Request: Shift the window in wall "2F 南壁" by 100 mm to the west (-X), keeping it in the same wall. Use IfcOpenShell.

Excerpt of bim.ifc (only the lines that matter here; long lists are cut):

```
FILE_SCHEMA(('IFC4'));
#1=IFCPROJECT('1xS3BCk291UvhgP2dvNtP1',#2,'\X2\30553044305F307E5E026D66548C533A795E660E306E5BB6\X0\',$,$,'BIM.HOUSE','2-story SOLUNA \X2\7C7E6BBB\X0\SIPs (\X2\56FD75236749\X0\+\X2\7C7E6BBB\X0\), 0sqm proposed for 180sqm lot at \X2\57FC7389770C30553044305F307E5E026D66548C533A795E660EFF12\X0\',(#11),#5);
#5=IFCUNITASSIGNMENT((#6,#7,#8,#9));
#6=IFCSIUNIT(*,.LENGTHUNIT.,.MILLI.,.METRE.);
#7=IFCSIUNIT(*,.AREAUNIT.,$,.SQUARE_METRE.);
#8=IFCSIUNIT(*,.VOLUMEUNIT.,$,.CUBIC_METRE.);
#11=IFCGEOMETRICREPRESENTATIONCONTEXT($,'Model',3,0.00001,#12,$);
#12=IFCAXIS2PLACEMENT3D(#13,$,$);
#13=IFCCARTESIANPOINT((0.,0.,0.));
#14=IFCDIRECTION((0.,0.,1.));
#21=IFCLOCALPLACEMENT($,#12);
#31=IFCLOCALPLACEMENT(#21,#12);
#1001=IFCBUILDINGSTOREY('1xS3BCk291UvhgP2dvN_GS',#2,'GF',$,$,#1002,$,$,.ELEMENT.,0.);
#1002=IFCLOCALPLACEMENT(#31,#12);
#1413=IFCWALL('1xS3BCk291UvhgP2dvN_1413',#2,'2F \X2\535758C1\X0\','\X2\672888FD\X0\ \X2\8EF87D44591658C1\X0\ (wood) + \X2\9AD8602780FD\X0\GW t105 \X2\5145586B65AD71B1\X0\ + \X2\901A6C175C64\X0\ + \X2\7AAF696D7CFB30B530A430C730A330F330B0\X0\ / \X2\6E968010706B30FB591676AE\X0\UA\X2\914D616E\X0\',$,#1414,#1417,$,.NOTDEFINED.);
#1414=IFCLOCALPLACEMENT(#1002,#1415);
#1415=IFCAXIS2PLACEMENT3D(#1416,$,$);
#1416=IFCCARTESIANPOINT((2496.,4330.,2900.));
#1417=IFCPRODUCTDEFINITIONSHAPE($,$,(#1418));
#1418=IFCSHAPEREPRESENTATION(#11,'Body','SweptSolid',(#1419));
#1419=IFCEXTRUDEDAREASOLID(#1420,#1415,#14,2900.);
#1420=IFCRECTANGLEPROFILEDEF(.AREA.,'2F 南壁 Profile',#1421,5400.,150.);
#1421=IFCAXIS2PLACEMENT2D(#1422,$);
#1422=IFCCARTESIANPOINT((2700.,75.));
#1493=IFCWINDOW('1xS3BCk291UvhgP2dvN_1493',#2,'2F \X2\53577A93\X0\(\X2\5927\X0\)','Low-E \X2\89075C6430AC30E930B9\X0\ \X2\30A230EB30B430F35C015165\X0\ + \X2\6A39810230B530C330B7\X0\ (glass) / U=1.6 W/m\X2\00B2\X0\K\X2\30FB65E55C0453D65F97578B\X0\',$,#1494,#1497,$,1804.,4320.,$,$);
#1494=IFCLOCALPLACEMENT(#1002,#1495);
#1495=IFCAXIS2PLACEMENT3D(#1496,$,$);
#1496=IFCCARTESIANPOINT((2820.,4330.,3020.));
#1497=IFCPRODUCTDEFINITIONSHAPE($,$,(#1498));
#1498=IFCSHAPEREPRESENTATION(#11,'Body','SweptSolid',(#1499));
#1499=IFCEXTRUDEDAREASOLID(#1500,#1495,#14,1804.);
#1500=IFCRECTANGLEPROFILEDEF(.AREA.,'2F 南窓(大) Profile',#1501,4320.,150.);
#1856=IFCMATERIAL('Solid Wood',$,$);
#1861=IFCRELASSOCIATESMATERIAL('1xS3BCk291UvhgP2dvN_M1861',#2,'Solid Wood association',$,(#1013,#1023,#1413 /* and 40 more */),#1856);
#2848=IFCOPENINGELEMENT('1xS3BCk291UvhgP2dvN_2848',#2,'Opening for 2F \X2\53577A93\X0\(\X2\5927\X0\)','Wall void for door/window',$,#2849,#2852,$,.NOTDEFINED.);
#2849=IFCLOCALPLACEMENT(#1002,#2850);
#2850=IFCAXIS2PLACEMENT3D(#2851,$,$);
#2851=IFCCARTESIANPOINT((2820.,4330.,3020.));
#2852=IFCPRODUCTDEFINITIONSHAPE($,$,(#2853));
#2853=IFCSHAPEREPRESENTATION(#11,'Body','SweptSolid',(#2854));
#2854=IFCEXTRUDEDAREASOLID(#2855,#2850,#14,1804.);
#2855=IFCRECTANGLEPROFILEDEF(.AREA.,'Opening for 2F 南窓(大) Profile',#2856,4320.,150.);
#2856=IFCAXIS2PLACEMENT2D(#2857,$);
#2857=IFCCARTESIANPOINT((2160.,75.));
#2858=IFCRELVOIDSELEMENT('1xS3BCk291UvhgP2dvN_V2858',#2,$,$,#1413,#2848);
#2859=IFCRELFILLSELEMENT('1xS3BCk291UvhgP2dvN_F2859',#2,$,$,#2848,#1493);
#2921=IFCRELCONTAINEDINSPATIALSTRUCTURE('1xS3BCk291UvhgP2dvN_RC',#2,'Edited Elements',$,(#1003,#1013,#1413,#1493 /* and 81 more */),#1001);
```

```python
import ifcopenshell
import ifcopenshell.api.geometry
import ifcopenshell.util.placement
import ifcopenshell.util.unit

model = ifcopenshell.open("bim.ifc")
unit_scale = ifcopenshell.util.unit.calculate_unit_scale(model)

window = model.by_id(1493)
opening = window.FillsVoids[0].RelatingOpeningElement
wall = opening.VoidsElements[0].RelatingBuildingElement

wall_matrix = ifcopenshell.util.placement.get_local_placement(wall.ObjectPlacement)
shift = wall_matrix[:3, 0] * -0.1 / unit_scale
before = ifcopenshell.util.placement.get_local_placement(window.ObjectPlacement)[:3, 3].copy()

# The window is not placed relative to its opening, so move both.
for product in (opening, window):
    matrix = ifcopenshell.util.placement.get_local_placement(product.ObjectPlacement)
    matrix[:3, 3] += shift
    ifcopenshell.api.geometry.edit_object_placement(model, product=product, matrix=matrix, is_si=False)

after = ifcopenshell.util.placement.get_local_placement(window.ObjectPlacement)[:3, 3]
print("window moved by", (after - before).round(3) + 0.0)

model.write("bim_rev.ifc")
```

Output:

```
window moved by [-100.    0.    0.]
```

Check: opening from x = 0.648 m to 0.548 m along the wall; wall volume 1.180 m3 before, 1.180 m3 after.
